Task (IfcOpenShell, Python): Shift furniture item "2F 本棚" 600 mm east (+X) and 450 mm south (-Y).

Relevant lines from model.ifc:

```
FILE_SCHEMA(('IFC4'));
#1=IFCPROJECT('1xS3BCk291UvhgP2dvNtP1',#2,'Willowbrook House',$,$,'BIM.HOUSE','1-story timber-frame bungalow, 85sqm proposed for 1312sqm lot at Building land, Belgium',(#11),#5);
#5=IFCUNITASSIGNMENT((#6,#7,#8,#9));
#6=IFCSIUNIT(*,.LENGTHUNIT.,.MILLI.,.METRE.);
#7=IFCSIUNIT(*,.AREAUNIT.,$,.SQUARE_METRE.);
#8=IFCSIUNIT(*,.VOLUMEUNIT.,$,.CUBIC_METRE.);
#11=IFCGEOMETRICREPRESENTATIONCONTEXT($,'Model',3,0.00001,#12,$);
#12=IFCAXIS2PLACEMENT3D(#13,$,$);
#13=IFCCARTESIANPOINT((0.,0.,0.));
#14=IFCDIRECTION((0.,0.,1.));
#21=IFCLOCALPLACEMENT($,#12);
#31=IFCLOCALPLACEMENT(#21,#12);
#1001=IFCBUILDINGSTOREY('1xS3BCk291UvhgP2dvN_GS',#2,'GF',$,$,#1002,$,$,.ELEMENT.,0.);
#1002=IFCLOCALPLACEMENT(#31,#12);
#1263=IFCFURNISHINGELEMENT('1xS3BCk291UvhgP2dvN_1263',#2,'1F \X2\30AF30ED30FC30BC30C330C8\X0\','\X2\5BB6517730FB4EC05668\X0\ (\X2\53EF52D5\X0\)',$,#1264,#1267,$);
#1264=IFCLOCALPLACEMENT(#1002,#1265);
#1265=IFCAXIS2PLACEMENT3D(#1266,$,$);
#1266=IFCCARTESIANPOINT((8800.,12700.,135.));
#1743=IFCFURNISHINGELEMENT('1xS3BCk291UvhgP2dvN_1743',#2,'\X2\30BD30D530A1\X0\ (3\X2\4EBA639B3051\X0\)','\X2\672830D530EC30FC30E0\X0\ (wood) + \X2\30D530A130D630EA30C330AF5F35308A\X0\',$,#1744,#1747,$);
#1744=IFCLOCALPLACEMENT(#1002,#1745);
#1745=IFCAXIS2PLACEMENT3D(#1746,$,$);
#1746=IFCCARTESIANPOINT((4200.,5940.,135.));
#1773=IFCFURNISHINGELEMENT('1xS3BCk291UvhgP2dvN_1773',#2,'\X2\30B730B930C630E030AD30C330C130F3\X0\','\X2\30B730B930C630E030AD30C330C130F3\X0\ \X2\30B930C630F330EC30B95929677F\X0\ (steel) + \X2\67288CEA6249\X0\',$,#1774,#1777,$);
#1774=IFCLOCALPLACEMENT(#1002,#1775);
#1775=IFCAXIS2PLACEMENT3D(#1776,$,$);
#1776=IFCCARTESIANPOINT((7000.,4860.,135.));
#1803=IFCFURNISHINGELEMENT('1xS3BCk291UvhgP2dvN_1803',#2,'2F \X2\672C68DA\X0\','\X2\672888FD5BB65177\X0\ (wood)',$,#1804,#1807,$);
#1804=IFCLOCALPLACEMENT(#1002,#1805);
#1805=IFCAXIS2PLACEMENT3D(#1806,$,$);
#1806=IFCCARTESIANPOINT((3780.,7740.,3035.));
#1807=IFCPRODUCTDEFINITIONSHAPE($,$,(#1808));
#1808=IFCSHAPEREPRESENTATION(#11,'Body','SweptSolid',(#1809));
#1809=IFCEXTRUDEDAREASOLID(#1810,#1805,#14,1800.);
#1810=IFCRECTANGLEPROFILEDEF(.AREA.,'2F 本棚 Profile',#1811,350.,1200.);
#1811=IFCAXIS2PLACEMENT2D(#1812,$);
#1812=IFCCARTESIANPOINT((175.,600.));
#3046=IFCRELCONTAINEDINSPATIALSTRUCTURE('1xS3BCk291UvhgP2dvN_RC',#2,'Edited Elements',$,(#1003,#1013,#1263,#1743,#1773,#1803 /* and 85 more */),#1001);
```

```python
import ifcopenshell
import ifcopenshell.api.geometry
import ifcopenshell.util.placement
import ifcopenshell.util.unit

model = ifcopenshell.open("model.ifc")
unit_scale = ifcopenshell.util.unit.calculate_unit_scale(model)

item = model.by_guid("1xS3BCk291UvhgP2dvN_1803")
matrix = ifcopenshell.util.placement.get_local_placement(item.ObjectPlacement)
matrix[0, 3] += 0.6 / unit_scale
matrix[1, 3] -= 0.45 / unit_scale
ifcopenshell.api.geometry.edit_object_placement(model, product=item, matrix=matrix, is_si=False)

print(ifcopenshell.util.placement.get_local_placement(item.ObjectPlacement).round(3) + 0.0)

model.write("model_edited.ifc")
```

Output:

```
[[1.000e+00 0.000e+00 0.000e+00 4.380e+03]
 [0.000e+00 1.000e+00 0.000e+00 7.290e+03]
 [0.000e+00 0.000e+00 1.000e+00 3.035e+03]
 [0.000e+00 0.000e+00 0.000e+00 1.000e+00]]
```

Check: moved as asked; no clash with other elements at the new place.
